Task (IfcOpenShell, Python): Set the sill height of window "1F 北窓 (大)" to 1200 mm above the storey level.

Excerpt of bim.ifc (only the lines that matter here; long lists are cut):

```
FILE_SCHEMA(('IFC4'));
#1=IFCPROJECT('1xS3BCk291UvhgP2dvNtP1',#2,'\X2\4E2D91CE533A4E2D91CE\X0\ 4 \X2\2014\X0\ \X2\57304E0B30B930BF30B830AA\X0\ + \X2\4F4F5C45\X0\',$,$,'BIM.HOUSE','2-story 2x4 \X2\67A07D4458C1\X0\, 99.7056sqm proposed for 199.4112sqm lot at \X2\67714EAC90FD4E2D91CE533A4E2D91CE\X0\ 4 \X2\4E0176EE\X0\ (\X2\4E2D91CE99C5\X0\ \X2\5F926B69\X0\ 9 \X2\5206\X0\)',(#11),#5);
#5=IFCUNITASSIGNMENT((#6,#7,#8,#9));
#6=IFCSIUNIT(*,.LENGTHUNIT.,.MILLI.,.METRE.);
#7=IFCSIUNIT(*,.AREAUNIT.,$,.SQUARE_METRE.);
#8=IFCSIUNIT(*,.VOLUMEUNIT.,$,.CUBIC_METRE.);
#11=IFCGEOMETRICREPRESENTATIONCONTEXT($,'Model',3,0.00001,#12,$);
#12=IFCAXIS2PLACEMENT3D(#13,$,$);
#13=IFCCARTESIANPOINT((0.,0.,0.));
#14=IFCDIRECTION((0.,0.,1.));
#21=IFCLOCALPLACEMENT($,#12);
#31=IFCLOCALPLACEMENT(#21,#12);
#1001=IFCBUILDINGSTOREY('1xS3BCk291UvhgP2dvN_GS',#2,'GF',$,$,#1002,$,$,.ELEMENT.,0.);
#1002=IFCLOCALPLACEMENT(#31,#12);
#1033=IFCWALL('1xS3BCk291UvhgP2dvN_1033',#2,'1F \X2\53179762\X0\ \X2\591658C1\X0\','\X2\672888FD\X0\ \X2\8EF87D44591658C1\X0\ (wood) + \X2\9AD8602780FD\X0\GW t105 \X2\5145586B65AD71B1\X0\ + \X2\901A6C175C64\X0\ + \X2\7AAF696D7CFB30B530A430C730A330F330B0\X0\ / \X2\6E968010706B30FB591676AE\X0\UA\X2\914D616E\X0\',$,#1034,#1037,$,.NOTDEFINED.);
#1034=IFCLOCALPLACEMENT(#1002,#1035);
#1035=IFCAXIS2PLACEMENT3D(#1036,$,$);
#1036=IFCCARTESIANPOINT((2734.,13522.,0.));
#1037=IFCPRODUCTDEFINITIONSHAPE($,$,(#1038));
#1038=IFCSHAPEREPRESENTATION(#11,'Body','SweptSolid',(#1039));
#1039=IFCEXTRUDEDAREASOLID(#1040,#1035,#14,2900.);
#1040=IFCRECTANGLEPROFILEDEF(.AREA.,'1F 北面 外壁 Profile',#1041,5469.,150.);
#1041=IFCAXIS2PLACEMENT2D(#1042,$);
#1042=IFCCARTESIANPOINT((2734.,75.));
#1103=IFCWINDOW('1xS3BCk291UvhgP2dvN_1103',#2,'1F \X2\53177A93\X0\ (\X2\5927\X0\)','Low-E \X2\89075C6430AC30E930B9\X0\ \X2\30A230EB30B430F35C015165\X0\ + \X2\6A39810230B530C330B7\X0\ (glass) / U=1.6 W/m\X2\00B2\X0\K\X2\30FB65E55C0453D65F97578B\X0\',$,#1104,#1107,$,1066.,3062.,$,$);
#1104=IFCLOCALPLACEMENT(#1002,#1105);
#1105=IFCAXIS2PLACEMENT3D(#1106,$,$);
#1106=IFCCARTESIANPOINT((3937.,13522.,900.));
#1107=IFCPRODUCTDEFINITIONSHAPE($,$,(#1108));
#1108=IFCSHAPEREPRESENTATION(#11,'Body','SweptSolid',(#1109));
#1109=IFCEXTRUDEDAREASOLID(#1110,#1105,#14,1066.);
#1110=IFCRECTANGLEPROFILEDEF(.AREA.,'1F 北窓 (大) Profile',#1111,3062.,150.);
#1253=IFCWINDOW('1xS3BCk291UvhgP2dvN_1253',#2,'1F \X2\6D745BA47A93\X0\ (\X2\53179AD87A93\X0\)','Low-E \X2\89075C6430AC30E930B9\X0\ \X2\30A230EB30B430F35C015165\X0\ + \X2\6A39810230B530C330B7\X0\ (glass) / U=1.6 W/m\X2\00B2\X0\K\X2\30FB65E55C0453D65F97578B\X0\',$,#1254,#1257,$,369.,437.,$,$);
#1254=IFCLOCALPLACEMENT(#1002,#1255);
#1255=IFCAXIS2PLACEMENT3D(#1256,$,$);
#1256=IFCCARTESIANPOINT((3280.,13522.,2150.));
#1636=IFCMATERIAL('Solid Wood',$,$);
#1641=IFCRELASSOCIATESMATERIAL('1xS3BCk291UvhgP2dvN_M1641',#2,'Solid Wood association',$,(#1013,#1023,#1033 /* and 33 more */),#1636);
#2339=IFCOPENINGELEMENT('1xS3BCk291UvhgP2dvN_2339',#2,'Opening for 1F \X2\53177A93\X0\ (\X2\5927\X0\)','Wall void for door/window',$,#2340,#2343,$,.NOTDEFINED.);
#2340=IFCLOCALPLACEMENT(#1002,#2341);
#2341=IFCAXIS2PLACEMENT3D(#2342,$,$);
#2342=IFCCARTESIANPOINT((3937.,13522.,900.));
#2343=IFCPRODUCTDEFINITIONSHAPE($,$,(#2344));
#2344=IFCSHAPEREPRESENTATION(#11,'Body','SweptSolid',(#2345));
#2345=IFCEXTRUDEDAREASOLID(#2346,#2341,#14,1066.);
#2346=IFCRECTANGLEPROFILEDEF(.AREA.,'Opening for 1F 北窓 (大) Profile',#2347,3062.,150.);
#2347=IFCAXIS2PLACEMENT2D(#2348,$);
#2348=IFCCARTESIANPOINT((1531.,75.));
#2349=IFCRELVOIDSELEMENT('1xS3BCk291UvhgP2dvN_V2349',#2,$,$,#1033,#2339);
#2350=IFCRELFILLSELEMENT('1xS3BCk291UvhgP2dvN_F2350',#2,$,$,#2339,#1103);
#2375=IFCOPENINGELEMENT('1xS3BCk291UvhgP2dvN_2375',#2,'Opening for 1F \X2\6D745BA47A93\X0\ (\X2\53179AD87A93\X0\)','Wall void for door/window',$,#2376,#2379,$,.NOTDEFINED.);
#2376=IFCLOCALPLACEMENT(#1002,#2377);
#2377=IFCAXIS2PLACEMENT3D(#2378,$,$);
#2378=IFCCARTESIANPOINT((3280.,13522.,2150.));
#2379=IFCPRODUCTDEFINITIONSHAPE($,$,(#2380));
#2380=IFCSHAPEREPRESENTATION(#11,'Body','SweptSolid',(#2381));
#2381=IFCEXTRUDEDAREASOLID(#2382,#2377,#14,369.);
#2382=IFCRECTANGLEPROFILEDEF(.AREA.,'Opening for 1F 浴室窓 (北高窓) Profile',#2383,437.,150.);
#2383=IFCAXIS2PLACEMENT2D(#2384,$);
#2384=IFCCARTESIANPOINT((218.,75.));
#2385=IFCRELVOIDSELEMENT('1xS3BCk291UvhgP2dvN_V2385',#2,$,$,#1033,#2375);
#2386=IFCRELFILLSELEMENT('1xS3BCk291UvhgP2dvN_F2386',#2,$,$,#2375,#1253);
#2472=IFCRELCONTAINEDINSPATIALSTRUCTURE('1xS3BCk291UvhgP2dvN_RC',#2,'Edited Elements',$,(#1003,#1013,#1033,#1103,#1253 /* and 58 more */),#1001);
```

```python
import numpy as np
import ifcopenshell
import ifcopenshell.api.geometry
import ifcopenshell.geom
import ifcopenshell.util.element
import ifcopenshell.util.placement
import ifcopenshell.util.shape
import ifcopenshell.util.unit

model = ifcopenshell.open("bim.ifc")
unit_scale = ifcopenshell.util.unit.calculate_unit_scale(model)

window = model.by_guid("1xS3BCk291UvhgP2dvN_1103")
opening = window.FillsVoids[0].RelatingOpeningElement
storey = ifcopenshell.util.element.get_container(window, ifc_class="IfcBuildingStorey")
level = ifcopenshell.util.placement.get_local_placement(storey.ObjectPlacement)[2, 3]

# The opening's origin need not be at the sill, so measure its lowest point.
shape = ifcopenshell.geom.create_shape(ifcopenshell.geom.settings(), opening)
bottom = ifcopenshell.util.shape.get_shape_bottom_elevation(shape, shape.geometry) / unit_scale
dz = level + 1.2 / unit_scale - bottom

shift = np.array([0.0, 0.0, dz])
# The window is not placed relative to its opening, so move both.
for product in (opening, window):
    matrix = ifcopenshell.util.placement.get_local_placement(product.ObjectPlacement)
    matrix[:3, 3] += shift
    ifcopenshell.api.geometry.edit_object_placement(model, product=product, matrix=matrix, is_si=False)

print(f"moved by {dz * unit_scale:+.3f} m")

model.write("bim_rev.ifc")
```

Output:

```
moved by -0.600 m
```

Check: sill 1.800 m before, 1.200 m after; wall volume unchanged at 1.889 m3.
